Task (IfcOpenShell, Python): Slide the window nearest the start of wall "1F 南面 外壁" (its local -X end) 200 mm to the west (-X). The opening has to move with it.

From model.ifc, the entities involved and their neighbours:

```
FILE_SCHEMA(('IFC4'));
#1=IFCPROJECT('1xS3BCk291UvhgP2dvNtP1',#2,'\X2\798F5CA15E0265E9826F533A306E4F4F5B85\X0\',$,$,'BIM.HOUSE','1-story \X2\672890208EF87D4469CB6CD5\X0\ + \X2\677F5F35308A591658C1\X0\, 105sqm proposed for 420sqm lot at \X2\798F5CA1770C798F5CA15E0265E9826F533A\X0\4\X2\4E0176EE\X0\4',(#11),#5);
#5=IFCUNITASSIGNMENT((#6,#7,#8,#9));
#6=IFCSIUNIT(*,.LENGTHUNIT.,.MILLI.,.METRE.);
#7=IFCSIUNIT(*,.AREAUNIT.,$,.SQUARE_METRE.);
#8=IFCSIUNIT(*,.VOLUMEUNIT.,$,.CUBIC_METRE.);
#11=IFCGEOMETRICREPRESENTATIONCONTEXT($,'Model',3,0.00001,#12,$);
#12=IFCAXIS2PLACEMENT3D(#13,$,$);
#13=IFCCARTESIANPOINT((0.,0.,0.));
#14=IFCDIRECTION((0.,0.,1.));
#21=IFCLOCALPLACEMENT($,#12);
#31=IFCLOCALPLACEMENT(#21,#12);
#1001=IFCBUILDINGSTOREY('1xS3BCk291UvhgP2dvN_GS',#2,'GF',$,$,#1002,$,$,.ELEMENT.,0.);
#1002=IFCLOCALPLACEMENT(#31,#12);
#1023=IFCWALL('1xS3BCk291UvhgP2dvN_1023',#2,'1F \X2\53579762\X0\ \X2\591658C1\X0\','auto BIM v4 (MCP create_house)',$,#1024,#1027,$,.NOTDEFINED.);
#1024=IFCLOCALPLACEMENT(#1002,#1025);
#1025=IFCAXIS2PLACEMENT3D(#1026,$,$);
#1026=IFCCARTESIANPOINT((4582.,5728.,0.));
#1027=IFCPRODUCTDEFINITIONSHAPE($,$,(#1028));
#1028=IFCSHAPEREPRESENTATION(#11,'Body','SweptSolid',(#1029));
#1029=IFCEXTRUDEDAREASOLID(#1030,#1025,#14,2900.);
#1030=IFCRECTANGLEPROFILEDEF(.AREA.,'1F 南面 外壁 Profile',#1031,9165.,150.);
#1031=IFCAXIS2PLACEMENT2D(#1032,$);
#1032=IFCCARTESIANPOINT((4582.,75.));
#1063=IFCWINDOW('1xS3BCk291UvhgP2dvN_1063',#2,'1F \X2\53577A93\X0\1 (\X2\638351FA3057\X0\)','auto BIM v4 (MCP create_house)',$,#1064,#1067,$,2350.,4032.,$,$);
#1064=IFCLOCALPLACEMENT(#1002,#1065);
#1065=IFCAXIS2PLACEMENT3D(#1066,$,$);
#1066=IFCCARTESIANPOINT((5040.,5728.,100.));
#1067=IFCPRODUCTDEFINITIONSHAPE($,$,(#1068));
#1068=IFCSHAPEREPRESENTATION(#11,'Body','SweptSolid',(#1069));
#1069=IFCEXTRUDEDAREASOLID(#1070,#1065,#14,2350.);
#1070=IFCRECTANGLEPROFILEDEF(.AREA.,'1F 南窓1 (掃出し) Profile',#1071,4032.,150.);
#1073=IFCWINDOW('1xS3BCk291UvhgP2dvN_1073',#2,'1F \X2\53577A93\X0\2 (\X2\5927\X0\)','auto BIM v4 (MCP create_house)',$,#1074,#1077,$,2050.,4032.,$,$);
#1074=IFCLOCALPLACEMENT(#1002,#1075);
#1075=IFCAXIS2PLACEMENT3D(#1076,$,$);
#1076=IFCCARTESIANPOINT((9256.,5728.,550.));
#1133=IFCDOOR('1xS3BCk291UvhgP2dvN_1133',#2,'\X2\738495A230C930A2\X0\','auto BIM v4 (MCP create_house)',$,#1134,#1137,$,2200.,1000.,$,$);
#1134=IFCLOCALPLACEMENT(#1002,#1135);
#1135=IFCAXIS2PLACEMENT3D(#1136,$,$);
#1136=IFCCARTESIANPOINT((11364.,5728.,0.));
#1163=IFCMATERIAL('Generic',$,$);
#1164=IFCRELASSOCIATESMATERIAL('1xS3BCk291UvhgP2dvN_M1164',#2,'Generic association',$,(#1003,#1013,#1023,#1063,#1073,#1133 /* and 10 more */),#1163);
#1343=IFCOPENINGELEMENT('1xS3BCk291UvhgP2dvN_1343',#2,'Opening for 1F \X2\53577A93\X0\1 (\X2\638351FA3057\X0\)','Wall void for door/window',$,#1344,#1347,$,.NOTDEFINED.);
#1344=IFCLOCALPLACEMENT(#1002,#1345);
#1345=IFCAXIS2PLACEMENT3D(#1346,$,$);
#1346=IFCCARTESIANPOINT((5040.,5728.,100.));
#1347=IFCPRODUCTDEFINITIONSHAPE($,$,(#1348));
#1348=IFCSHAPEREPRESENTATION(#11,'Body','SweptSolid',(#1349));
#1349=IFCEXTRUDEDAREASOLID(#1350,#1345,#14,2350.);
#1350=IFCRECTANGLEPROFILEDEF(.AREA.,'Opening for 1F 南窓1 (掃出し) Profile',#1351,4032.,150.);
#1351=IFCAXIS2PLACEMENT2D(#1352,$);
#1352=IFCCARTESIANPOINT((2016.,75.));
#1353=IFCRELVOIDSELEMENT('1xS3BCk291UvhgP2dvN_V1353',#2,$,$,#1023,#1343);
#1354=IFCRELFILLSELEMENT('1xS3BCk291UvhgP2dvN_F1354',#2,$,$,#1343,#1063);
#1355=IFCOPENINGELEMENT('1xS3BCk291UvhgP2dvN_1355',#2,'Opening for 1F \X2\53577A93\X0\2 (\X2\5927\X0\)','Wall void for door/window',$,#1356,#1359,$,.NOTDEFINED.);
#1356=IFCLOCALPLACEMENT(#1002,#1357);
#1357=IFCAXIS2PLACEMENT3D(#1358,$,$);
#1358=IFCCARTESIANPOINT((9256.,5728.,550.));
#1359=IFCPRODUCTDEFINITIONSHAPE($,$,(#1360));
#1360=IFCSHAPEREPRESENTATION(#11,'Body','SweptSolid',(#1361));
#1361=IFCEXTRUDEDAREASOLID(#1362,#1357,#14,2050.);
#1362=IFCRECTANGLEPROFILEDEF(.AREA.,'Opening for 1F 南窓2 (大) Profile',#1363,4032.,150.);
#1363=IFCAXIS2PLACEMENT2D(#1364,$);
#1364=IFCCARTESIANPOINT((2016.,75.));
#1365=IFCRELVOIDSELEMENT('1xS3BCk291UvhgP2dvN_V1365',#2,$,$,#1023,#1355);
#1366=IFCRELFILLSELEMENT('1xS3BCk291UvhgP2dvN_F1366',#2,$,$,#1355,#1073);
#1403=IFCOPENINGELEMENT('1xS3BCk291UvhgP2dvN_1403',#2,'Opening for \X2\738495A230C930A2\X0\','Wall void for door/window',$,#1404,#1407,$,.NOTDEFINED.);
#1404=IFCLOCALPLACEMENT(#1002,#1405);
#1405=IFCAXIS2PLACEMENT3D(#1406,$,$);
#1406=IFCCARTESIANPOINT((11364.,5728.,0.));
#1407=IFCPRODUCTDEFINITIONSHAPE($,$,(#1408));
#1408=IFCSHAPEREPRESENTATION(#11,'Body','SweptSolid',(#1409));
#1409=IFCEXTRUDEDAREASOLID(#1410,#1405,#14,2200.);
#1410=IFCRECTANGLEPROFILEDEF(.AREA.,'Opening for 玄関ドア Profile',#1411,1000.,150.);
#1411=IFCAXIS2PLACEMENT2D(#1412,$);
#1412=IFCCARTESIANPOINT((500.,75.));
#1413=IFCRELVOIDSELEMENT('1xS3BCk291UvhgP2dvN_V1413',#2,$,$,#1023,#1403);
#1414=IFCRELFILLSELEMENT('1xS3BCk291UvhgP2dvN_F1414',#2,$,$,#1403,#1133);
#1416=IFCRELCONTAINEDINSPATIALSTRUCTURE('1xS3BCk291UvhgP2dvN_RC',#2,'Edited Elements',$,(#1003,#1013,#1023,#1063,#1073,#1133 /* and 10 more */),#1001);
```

```python
import ifcopenshell
import ifcopenshell.api.geometry
import ifcopenshell.util.placement
import ifcopenshell.util.unit

model = ifcopenshell.open("model.ifc")
unit_scale = ifcopenshell.util.unit.calculate_unit_scale(model)

window = model.by_guid("1xS3BCk291UvhgP2dvN_1063")
opening = window.FillsVoids[0].RelatingOpeningElement
wall = opening.VoidsElements[0].RelatingBuildingElement

wall_matrix = ifcopenshell.util.placement.get_local_placement(wall.ObjectPlacement)
shift = wall_matrix[:3, 0] * -0.2 / unit_scale
before = ifcopenshell.util.placement.get_local_placement(window.ObjectPlacement)[:3, 3].copy()

# The window is not placed relative to its opening, so move both.
for product in (opening, window):
    matrix = ifcopenshell.util.placement.get_local_placement(product.ObjectPlacement)
    matrix[:3, 3] += shift
    ifcopenshell.api.geometry.edit_object_placement(model, product=product, matrix=matrix, is_si=False)

after = ifcopenshell.util.placement.get_local_placement(window.ObjectPlacement)[:3, 3]
print("window moved by", (after - before).round(3) + 0.0)

model.write("model_edited.ifc")
```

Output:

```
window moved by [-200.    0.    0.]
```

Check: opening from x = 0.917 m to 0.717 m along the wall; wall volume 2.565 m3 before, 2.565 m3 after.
